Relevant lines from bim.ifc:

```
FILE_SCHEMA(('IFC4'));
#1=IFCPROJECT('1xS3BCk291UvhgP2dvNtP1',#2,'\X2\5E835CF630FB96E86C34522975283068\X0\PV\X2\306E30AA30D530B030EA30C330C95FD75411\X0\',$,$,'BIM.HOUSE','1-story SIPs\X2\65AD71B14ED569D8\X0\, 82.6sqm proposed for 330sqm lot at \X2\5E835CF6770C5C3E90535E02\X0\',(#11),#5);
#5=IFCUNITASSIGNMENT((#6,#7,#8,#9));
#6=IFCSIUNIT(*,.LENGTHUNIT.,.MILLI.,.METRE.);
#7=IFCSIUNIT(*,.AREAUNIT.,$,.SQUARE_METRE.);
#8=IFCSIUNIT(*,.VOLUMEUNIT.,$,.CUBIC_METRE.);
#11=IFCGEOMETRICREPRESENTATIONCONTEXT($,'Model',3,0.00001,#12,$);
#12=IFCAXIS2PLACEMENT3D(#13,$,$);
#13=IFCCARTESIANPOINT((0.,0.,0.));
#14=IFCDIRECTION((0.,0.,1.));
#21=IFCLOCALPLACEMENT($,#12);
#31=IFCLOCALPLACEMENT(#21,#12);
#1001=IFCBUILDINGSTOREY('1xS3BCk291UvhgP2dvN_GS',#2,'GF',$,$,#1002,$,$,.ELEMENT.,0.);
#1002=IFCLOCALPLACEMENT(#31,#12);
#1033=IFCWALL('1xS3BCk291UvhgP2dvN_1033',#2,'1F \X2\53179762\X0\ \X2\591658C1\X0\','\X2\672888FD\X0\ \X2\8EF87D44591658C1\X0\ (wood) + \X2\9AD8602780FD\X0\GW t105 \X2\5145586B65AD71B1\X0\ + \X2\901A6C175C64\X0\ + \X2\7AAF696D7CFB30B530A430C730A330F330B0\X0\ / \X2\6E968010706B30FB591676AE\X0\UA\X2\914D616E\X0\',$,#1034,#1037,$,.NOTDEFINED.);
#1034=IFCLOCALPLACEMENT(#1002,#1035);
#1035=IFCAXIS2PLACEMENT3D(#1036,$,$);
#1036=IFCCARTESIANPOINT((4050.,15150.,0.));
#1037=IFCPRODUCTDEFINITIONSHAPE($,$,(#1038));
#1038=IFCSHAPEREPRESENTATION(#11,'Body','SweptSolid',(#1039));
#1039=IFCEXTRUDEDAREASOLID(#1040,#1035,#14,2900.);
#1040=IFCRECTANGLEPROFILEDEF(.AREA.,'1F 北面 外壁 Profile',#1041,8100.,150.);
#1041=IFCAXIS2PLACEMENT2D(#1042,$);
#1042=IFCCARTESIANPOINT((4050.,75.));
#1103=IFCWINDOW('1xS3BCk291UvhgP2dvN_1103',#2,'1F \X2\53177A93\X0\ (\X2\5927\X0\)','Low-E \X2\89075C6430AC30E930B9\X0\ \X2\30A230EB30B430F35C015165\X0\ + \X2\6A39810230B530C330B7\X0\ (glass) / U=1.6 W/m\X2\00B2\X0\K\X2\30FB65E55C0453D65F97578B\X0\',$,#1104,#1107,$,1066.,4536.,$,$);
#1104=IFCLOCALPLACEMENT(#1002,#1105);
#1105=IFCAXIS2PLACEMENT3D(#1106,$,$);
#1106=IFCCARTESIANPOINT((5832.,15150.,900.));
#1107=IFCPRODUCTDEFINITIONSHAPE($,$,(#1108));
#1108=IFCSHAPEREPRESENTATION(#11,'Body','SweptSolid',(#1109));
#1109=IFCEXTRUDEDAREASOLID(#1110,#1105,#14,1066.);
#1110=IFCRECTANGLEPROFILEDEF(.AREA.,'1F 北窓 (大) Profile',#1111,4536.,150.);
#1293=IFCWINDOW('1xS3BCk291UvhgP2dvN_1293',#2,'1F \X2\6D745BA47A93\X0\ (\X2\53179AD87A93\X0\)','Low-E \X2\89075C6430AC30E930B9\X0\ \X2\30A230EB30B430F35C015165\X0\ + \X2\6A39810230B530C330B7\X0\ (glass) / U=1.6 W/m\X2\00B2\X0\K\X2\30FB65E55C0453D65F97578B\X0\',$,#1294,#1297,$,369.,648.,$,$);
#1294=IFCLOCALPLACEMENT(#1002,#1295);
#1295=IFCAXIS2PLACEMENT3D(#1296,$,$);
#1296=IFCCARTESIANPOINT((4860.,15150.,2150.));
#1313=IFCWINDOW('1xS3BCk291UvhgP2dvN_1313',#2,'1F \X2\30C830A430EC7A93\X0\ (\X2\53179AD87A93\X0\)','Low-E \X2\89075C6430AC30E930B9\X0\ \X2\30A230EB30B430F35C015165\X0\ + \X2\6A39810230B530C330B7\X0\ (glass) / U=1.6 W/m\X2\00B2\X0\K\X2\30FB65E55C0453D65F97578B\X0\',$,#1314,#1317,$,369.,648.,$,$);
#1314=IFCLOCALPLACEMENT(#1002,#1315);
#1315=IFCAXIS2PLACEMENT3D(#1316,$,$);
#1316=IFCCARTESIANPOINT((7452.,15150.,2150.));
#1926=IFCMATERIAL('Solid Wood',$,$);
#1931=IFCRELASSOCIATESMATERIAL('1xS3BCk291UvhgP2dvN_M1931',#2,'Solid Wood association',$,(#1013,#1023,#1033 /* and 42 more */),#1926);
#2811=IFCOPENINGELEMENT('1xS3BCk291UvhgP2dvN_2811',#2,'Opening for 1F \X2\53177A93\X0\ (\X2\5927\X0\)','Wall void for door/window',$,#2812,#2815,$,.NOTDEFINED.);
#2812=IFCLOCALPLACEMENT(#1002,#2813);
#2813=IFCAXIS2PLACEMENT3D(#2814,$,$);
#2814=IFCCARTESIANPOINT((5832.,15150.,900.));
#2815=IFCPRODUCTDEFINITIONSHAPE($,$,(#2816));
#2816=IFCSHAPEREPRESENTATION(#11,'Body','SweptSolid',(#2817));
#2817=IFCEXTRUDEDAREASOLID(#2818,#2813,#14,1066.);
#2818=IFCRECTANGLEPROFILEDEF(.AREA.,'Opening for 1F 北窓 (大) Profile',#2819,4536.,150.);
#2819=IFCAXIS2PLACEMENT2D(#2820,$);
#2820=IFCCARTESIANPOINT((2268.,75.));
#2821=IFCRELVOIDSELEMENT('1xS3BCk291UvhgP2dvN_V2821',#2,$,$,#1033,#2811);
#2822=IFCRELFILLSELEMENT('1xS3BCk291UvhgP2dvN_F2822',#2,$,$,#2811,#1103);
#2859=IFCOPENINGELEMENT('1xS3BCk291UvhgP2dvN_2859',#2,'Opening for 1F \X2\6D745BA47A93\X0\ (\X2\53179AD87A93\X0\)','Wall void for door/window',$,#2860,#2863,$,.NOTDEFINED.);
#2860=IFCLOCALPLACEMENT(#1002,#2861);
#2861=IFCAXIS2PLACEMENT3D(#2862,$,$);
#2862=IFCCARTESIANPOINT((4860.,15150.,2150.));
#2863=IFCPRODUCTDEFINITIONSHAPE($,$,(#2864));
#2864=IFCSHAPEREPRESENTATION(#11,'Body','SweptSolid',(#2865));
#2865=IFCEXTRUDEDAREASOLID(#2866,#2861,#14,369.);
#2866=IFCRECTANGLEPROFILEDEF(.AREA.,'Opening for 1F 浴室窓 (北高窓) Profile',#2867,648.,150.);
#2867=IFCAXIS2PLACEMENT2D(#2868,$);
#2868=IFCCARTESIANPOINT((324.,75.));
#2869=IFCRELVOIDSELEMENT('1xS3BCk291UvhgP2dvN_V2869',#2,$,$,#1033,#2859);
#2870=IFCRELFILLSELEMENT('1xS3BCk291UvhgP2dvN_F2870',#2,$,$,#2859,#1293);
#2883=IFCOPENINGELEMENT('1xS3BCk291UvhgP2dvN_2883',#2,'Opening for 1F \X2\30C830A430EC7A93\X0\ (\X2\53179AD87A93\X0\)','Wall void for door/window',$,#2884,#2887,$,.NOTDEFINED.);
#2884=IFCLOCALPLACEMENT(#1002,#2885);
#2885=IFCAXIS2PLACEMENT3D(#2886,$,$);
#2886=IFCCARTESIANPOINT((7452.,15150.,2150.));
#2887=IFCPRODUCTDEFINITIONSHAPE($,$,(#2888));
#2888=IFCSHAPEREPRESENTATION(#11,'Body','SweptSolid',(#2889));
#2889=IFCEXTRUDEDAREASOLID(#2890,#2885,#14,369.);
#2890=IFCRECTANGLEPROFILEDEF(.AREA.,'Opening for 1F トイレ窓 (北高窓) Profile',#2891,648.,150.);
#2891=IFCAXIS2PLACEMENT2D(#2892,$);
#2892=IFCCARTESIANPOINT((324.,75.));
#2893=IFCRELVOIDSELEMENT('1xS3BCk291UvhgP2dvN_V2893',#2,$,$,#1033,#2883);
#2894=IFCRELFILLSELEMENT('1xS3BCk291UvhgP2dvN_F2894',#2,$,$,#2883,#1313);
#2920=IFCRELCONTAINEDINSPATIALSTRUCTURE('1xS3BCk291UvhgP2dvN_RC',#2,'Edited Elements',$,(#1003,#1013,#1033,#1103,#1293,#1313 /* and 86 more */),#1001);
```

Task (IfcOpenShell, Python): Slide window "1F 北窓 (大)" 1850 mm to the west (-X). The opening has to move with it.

```python
import ifcopenshell
import ifcopenshell.api.geometry
import ifcopenshell.util.placement

model = ifcopenshell.open("bim.ifc")

window = model.by_guid("1xS3BCk291UvhgP2dvN_1103")
opening = window.FillsVoids[0].RelatingOpeningElement
wall = opening.VoidsElements[0].RelatingBuildingElement

wall_matrix = ifcopenshell.util.placement.get_local_placement(wall.ObjectPlacement)
shift = wall_matrix[:3, 0] * -1850.0
before = ifcopenshell.util.placement.get_local_placement(window.ObjectPlacement)[:3, 3].copy()

# The window is not placed relative to its opening, so move both.
for product in (opening, window):
    matrix = ifcopenshell.util.placement.get_local_placement(product.ObjectPlacement)
    matrix[:3, 3] += shift
    ifcopenshell.api.geometry.edit_object_placement(model, product=product, matrix=matrix, is_si=False)

after = ifcopenshell.util.placement.get_local_placement(window.ObjectPlacement)[:3, 3]
print("window moved by", (after - before).round(3) + 0.0)

model.write("bim_rev.ifc")
```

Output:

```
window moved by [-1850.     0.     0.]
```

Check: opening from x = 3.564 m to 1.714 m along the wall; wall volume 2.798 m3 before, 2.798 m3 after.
